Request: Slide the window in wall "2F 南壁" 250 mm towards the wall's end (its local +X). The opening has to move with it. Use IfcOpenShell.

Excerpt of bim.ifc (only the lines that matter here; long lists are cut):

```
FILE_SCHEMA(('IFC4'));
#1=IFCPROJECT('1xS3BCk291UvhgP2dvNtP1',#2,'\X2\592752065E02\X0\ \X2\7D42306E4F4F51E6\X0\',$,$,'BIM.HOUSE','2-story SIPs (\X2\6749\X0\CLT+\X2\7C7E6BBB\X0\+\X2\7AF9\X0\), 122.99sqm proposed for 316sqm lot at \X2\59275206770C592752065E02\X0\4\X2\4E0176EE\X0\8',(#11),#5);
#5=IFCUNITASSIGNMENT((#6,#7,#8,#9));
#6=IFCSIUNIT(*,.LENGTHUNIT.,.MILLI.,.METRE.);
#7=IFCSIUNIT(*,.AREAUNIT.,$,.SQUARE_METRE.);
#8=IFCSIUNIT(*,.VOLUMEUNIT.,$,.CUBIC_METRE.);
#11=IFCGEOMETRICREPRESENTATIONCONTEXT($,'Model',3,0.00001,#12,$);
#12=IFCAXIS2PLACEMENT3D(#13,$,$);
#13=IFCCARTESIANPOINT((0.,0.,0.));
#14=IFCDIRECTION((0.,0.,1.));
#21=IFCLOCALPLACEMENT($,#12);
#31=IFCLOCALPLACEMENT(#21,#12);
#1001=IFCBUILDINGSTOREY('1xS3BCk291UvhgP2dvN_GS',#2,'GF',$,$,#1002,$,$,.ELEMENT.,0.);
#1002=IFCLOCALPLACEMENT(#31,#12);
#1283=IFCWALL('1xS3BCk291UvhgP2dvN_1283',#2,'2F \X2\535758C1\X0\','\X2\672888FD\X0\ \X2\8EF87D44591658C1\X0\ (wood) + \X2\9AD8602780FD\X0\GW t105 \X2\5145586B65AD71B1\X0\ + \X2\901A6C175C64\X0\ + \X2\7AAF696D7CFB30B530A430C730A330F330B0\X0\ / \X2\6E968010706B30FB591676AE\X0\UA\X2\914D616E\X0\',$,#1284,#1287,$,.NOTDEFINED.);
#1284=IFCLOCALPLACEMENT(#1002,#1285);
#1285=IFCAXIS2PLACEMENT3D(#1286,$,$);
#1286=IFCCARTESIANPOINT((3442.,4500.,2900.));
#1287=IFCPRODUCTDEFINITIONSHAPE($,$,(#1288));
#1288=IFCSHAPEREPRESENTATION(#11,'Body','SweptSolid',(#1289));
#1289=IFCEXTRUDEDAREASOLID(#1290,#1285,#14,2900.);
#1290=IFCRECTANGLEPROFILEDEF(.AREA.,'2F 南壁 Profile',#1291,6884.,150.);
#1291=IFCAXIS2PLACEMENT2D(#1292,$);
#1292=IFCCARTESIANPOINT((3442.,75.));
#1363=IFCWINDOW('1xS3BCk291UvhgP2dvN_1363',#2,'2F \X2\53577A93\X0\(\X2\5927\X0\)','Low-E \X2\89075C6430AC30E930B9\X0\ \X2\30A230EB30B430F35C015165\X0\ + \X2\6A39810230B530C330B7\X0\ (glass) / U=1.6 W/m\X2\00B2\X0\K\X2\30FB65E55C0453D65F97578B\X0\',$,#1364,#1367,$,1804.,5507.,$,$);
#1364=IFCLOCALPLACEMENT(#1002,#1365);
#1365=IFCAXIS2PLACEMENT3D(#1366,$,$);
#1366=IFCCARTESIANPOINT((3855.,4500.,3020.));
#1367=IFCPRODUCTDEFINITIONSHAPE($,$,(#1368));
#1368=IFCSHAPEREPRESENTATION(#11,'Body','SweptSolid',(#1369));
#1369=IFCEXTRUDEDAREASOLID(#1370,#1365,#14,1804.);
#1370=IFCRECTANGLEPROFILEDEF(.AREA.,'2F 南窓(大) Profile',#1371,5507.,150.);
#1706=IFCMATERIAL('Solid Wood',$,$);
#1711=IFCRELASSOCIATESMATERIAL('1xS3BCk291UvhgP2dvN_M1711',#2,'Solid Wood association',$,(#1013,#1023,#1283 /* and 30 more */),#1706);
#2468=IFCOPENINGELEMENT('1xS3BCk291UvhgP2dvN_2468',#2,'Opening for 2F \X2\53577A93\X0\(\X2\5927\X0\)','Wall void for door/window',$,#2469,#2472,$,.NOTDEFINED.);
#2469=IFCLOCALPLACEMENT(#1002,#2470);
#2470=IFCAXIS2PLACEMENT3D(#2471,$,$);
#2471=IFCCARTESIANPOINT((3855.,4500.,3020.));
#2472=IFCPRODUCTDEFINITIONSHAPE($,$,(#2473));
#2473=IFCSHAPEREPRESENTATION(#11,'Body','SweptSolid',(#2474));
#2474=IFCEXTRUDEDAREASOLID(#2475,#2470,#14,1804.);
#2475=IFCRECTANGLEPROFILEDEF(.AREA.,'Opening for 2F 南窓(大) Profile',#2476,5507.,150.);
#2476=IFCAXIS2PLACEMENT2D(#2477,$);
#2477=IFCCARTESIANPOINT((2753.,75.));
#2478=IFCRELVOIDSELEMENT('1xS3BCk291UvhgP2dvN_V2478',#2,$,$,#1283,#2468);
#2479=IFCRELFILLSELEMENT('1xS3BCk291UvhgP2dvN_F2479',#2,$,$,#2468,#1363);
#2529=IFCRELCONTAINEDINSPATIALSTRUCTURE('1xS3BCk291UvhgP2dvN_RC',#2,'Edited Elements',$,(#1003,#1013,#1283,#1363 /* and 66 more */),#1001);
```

```python
import ifcopenshell
import ifcopenshell.api.geometry
import ifcopenshell.util.placement
import ifcopenshell.util.unit

model = ifcopenshell.open("bim.ifc")
unit_scale = ifcopenshell.util.unit.calculate_unit_scale(model)

window = model.by_guid("1xS3BCk291UvhgP2dvN_1363")
opening = window.FillsVoids[0].RelatingOpeningElement
wall = opening.VoidsElements[0].RelatingBuildingElement

wall_matrix = ifcopenshell.util.placement.get_local_placement(wall.ObjectPlacement)
shift = wall_matrix[:3, 0] * 0.25 / unit_scale
before = ifcopenshell.util.placement.get_local_placement(window.ObjectPlacement)[:3, 3].copy()

# The window is not placed relative to its opening, so move both.
for product in (opening, window):
    matrix = ifcopenshell.util.placement.get_local_placement(product.ObjectPlacement)
    matrix[:3, 3] += shift
    ifcopenshell.api.geometry.edit_object_placement(model, product=product, matrix=matrix, is_si=False)

after = ifcopenshell.util.placement.get_local_placement(window.ObjectPlacement)[:3, 3]
print("window moved by", (after - before).round(3) + 0.0)

model.write("bim_updated.ifc")
```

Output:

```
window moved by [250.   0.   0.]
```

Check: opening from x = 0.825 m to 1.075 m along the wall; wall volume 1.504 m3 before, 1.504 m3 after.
